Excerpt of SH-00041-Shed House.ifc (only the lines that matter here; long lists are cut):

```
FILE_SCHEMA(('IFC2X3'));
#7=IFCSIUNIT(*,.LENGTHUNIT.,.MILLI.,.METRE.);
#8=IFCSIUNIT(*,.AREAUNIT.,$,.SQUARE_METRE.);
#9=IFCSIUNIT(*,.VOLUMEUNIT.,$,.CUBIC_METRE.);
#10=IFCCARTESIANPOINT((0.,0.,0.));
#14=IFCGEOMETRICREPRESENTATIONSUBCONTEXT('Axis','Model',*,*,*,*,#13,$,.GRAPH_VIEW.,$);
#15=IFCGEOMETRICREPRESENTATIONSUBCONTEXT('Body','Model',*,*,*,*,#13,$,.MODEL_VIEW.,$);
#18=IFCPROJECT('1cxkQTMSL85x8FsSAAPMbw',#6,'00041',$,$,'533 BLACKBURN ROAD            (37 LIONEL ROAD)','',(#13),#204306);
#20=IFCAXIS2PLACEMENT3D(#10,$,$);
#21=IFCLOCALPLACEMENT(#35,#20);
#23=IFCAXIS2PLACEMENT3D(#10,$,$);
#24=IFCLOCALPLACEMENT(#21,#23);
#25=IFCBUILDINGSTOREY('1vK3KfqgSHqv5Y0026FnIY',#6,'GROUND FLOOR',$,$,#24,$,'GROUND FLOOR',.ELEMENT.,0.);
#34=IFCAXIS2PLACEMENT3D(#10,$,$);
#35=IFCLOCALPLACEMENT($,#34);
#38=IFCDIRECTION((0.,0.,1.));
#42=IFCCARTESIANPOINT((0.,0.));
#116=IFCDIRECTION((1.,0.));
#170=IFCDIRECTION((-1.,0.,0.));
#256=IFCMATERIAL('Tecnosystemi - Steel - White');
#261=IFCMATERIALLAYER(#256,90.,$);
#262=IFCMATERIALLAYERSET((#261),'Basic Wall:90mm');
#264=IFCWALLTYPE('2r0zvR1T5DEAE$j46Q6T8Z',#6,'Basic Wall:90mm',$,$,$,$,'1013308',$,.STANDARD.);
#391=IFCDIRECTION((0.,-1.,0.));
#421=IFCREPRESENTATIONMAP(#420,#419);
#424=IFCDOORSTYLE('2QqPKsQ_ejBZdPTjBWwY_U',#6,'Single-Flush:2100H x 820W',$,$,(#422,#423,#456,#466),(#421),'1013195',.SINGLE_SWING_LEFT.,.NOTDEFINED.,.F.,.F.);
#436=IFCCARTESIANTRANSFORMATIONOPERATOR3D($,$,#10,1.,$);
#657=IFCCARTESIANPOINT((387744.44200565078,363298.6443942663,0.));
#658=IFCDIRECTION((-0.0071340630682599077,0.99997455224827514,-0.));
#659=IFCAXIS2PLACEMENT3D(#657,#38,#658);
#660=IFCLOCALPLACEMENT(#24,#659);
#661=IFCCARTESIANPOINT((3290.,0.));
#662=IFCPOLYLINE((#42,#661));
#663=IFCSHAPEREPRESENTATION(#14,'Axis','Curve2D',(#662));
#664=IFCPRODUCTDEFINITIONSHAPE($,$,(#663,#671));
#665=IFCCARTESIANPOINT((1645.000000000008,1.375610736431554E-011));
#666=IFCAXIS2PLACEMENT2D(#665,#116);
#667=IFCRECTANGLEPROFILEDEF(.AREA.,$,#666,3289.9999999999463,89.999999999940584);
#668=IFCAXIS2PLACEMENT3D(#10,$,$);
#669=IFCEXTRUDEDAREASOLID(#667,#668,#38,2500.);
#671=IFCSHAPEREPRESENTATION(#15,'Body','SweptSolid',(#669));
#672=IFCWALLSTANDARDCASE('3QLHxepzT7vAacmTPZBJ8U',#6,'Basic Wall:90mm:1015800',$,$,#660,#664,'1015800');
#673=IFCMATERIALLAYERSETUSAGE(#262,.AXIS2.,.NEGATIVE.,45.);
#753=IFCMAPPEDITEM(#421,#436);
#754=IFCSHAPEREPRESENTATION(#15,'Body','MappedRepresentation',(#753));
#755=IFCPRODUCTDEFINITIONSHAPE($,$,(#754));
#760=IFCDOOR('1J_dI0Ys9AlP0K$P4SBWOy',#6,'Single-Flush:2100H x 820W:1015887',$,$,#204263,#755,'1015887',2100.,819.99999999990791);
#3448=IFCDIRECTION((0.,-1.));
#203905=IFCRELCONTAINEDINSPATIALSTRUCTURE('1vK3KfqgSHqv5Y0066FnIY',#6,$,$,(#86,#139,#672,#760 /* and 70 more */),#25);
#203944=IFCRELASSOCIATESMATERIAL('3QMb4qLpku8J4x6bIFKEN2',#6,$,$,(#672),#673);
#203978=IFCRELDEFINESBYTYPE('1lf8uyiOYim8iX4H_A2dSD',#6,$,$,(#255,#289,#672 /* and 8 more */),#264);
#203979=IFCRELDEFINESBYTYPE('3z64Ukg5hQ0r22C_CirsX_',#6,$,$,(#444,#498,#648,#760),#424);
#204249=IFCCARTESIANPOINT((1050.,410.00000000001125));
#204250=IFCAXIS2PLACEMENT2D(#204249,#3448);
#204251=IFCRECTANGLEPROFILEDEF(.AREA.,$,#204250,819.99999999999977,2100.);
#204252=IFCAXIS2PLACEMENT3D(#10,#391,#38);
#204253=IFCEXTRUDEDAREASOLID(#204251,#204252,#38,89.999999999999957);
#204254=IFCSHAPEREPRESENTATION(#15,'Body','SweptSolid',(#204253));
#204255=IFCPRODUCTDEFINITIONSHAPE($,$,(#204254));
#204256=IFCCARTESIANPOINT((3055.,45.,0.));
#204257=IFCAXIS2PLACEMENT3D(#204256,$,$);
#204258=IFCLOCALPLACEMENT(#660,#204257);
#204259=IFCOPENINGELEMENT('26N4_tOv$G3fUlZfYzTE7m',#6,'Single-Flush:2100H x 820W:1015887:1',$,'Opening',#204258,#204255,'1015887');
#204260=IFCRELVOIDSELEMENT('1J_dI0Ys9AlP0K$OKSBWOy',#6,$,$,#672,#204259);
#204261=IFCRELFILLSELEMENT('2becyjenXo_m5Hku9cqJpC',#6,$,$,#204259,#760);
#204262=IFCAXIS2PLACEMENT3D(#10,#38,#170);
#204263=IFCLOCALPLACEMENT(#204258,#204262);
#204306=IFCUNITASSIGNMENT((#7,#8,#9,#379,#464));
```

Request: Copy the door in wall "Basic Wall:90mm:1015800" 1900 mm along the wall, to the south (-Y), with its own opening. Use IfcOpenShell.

```python
import ifcopenshell
import ifcopenshell.api.feature
import ifcopenshell.api.geometry
import ifcopenshell.api.root
import ifcopenshell.geom
import ifcopenshell.util.element
import ifcopenshell.util.placement
import ifcopenshell.util.shape

model = ifcopenshell.open("SH-00041-Shed House.ifc")
settings = ifcopenshell.geom.settings()


def volume(element):
    """Net volume in cubic metres, openings subtracted."""
    shape = ifcopenshell.geom.create_shape(settings, element)
    return ifcopenshell.util.shape.get_volume(shape.geometry)


def reuse_history(source, copy):
    """copy_class also copies each property set's owner history, people and application; keep the originals."""
    for rel in copy.IsDefinedBy:
        if rel.is_a("IfcRelDefinesByProperties") and (history := rel.RelatingPropertyDefinition.OwnerHistory):
            rel.RelatingPropertyDefinition.OwnerHistory = source.OwnerHistory
            ifcopenshell.util.element.remove_deep2(model, history)


door = model.by_guid("1J_dI0Ys9AlP0K$P4SBWOy")
opening = door.FillsVoids[0].RelatingOpeningElement
wall = opening.VoidsElements[0].RelatingBuildingElement
before = volume(wall)
shift = ifcopenshell.util.placement.get_local_placement(wall.ObjectPlacement)[:3, 0] * -1900.0

# copy_class copies the void relationship, type, container and properties, but no geometry.
new_opening = ifcopenshell.api.root.copy_class(model, product=opening)
new_opening.Representation = ifcopenshell.util.element.copy_deep(
    model, opening.Representation, exclude=["IfcGeometricRepresentationContext", "IfcRepresentationMap"]
)
new_opening.Name = "Single-Flush:2100H x 820W"
new_opening.Tag = None
new_door = ifcopenshell.api.root.copy_class(model, product=door)
new_door.Representation = ifcopenshell.util.element.copy_deep(
    model, door.Representation, exclude=["IfcGeometricRepresentationContext", "IfcRepresentationMap"]
)
new_door.Name = "Single-Flush:2100H x 820W"
new_door.Tag = None
reuse_history(door, new_door)
fills = ifcopenshell.api.feature.add_filling(model, opening=new_opening, element=new_door)
fills.OwnerHistory = new_door.OwnerHistory  # required in IFC2X3

for old, new in ((opening, new_opening), (door, new_door)):
    matrix = ifcopenshell.util.placement.get_local_placement(old.ObjectPlacement)
    matrix[:3, 3] += shift
    ifcopenshell.api.geometry.edit_object_placement(model, product=new, matrix=matrix, is_si=False)

after = volume(wall)

print(f"wall volume {before:.3f} -> {after:.3f} m3")

model.write("SH-00041-Shed House_rev.ifc")
```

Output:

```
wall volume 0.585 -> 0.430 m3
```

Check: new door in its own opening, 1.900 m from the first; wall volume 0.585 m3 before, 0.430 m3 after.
